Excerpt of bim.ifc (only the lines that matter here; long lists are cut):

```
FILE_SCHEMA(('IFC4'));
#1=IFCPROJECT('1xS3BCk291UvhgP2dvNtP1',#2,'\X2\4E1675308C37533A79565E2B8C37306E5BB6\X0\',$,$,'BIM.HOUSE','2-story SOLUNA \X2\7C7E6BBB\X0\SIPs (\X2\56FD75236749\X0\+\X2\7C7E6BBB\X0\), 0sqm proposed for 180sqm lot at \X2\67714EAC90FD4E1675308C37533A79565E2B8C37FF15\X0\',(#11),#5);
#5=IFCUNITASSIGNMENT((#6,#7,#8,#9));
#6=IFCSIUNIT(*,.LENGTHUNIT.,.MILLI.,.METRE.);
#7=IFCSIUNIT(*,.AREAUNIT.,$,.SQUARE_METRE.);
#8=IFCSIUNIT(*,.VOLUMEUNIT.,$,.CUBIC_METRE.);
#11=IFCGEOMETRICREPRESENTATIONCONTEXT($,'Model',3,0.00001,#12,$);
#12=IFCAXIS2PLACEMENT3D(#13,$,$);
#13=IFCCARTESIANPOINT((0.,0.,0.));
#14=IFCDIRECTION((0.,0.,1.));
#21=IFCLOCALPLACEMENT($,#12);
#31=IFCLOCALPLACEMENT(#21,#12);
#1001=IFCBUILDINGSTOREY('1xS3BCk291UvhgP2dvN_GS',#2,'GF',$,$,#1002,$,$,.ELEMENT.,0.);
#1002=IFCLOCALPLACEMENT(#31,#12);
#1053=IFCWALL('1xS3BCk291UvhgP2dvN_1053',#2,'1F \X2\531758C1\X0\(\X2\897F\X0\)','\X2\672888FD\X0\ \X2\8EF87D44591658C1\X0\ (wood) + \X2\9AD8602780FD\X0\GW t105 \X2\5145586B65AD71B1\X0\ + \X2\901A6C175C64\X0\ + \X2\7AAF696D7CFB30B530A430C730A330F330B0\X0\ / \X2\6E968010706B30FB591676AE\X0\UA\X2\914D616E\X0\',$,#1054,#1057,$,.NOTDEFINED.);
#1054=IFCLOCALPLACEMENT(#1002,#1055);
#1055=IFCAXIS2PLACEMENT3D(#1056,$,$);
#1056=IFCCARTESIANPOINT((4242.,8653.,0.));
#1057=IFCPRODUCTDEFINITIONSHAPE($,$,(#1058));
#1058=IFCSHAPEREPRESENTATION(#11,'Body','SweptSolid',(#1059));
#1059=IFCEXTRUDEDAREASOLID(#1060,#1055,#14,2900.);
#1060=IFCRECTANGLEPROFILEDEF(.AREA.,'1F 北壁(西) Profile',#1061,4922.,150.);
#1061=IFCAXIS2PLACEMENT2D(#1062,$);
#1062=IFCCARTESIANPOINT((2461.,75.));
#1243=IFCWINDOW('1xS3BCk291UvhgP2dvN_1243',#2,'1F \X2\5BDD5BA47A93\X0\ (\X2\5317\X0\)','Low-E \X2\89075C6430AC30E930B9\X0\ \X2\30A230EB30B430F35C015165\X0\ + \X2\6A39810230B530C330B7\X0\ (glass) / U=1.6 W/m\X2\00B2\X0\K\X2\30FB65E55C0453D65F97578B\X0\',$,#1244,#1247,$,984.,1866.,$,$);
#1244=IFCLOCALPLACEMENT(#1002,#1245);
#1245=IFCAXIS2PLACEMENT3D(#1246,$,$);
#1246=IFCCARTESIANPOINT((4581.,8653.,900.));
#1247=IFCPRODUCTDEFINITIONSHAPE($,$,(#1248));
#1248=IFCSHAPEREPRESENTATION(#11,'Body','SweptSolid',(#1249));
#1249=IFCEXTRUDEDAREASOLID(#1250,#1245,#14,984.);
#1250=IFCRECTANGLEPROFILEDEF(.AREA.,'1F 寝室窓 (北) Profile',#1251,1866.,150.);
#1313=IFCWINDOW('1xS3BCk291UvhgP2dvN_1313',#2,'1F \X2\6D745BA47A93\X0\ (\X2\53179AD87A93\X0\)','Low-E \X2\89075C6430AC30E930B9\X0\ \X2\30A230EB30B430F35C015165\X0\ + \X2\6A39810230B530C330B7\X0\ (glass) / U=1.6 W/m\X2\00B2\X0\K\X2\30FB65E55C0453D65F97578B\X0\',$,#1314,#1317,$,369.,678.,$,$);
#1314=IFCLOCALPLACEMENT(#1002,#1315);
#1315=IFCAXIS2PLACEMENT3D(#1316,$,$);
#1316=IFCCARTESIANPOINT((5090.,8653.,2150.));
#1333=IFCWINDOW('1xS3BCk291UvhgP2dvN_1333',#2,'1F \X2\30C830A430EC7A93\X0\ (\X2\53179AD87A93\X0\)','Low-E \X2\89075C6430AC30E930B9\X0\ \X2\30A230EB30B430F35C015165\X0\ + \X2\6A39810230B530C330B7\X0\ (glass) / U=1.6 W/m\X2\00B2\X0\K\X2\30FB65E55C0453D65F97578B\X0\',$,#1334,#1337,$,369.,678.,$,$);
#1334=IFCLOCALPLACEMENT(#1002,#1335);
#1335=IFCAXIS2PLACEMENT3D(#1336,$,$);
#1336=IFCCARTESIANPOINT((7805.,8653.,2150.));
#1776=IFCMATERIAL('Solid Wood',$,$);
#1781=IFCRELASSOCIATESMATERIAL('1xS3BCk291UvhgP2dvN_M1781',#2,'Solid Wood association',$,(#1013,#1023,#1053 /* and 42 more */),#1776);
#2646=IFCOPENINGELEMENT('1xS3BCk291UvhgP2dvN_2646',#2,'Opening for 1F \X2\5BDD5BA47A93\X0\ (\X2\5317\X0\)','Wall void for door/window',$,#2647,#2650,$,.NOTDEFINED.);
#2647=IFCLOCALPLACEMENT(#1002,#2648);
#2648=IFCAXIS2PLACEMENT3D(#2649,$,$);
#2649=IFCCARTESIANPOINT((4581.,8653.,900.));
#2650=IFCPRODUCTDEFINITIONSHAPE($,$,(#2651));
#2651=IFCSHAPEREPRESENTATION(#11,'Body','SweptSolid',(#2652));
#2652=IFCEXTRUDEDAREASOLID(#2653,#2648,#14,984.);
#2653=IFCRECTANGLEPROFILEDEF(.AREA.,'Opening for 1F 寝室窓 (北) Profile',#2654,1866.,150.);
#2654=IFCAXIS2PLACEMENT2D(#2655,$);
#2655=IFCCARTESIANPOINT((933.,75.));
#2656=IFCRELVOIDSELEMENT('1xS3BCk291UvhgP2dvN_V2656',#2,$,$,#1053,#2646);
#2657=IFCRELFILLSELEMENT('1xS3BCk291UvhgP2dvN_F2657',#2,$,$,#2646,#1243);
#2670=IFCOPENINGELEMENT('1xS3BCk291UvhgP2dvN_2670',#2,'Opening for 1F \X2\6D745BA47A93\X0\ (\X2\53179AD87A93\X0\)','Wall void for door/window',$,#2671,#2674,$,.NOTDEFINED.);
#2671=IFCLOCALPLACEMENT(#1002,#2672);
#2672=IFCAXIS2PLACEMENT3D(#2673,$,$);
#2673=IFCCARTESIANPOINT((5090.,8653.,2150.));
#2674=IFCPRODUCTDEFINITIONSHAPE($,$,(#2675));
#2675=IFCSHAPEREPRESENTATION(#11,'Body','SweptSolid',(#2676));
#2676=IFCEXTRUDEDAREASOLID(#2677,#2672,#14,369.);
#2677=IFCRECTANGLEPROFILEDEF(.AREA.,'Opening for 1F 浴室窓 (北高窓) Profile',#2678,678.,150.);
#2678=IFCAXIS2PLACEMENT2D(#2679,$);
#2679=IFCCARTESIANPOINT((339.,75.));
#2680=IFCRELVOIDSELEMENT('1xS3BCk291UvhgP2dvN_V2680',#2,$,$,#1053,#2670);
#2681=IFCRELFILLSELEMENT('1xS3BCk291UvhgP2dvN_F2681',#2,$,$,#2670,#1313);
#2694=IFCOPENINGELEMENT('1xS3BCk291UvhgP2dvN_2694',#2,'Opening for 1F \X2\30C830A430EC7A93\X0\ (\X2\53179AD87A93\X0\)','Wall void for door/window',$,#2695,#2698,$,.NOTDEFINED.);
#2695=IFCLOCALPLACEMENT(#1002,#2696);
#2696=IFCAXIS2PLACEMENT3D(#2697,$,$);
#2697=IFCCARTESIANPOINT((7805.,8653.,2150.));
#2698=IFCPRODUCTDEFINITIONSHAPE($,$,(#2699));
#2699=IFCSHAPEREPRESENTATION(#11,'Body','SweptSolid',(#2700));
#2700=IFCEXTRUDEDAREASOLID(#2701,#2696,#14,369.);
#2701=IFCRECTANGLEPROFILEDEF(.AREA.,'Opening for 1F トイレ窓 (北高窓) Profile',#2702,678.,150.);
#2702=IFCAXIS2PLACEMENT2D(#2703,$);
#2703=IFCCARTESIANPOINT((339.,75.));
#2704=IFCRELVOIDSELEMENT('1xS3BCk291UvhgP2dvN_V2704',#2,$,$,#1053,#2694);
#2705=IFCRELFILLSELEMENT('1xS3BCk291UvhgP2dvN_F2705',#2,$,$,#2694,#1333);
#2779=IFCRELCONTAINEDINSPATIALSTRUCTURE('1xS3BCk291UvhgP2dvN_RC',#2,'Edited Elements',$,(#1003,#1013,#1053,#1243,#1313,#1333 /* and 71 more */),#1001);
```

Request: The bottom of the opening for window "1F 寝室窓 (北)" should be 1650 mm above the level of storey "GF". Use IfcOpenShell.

```python
import numpy as np
import ifcopenshell
import ifcopenshell.api.geometry
import ifcopenshell.geom
import ifcopenshell.util.element
import ifcopenshell.util.placement
import ifcopenshell.util.shape
import ifcopenshell.util.unit

model = ifcopenshell.open("bim.ifc")
unit_scale = ifcopenshell.util.unit.calculate_unit_scale(model)

window = model.by_guid("1xS3BCk291UvhgP2dvN_1243")
opening = window.FillsVoids[0].RelatingOpeningElement
storey = ifcopenshell.util.element.get_container(window, ifc_class="IfcBuildingStorey")
level = ifcopenshell.util.placement.get_local_placement(storey.ObjectPlacement)[2, 3]

# The opening's origin need not be at the sill, so measure its lowest point.
shape = ifcopenshell.geom.create_shape(ifcopenshell.geom.settings(), opening)
bottom = ifcopenshell.util.shape.get_shape_bottom_elevation(shape, shape.geometry) / unit_scale
dz = level + 1650.0 - bottom

shift = np.array([0.0, 0.0, dz])
# The window is not placed relative to its opening, so move both.
for product in (opening, window):
    matrix = ifcopenshell.util.placement.get_local_placement(product.ObjectPlacement)
    matrix[:3, 3] += shift
    ifcopenshell.api.geometry.edit_object_placement(model, product=product, matrix=matrix, is_si=False)

print(f"moved by {dz * unit_scale:+.3f} m")

model.write("bim_rev.ifc")
```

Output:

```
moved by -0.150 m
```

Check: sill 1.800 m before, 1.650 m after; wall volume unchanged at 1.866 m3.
